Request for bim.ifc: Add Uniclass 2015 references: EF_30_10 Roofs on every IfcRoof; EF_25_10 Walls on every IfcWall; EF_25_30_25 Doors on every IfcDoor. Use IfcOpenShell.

First a look at what the model holds.

```python
import ifcopenshell

model = ifcopenshell.open("bim.ifc")
print(model.schema)
print("classifications:", [c.Name for c in model.by_type("IfcClassification")])
for ifc_class in ("IfcDoor", "IfcRoof", "IfcStair", "IfcWall", "IfcWindow"):
    print(ifc_class, len(model.by_type(ifc_class)))
```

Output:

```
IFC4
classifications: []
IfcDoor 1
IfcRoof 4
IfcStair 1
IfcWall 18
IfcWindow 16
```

```python
import ifcopenshell
import ifcopenshell.api.classification

model = ifcopenshell.open("bim.ifc")

system = ifcopenshell.api.classification.add_classification(model, classification="Uniclass 2015")

codes = {
    "IfcRoof": ("EF_30_10", "Roofs"),
    "IfcWall": ("EF_25_10", "Walls"),
    "IfcDoor": ("EF_25_30_25", "Doors"),
}
for ifc_class, (code, name) in codes.items():
    products = model.by_type(ifc_class)
    ifcopenshell.api.classification.add_reference(
        model, products=products, classification=system, identification=code, name=name
    )
    print(code, len(products))

model.write("bim_updated.ifc")
```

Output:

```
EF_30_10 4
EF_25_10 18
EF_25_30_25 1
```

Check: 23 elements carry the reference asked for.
